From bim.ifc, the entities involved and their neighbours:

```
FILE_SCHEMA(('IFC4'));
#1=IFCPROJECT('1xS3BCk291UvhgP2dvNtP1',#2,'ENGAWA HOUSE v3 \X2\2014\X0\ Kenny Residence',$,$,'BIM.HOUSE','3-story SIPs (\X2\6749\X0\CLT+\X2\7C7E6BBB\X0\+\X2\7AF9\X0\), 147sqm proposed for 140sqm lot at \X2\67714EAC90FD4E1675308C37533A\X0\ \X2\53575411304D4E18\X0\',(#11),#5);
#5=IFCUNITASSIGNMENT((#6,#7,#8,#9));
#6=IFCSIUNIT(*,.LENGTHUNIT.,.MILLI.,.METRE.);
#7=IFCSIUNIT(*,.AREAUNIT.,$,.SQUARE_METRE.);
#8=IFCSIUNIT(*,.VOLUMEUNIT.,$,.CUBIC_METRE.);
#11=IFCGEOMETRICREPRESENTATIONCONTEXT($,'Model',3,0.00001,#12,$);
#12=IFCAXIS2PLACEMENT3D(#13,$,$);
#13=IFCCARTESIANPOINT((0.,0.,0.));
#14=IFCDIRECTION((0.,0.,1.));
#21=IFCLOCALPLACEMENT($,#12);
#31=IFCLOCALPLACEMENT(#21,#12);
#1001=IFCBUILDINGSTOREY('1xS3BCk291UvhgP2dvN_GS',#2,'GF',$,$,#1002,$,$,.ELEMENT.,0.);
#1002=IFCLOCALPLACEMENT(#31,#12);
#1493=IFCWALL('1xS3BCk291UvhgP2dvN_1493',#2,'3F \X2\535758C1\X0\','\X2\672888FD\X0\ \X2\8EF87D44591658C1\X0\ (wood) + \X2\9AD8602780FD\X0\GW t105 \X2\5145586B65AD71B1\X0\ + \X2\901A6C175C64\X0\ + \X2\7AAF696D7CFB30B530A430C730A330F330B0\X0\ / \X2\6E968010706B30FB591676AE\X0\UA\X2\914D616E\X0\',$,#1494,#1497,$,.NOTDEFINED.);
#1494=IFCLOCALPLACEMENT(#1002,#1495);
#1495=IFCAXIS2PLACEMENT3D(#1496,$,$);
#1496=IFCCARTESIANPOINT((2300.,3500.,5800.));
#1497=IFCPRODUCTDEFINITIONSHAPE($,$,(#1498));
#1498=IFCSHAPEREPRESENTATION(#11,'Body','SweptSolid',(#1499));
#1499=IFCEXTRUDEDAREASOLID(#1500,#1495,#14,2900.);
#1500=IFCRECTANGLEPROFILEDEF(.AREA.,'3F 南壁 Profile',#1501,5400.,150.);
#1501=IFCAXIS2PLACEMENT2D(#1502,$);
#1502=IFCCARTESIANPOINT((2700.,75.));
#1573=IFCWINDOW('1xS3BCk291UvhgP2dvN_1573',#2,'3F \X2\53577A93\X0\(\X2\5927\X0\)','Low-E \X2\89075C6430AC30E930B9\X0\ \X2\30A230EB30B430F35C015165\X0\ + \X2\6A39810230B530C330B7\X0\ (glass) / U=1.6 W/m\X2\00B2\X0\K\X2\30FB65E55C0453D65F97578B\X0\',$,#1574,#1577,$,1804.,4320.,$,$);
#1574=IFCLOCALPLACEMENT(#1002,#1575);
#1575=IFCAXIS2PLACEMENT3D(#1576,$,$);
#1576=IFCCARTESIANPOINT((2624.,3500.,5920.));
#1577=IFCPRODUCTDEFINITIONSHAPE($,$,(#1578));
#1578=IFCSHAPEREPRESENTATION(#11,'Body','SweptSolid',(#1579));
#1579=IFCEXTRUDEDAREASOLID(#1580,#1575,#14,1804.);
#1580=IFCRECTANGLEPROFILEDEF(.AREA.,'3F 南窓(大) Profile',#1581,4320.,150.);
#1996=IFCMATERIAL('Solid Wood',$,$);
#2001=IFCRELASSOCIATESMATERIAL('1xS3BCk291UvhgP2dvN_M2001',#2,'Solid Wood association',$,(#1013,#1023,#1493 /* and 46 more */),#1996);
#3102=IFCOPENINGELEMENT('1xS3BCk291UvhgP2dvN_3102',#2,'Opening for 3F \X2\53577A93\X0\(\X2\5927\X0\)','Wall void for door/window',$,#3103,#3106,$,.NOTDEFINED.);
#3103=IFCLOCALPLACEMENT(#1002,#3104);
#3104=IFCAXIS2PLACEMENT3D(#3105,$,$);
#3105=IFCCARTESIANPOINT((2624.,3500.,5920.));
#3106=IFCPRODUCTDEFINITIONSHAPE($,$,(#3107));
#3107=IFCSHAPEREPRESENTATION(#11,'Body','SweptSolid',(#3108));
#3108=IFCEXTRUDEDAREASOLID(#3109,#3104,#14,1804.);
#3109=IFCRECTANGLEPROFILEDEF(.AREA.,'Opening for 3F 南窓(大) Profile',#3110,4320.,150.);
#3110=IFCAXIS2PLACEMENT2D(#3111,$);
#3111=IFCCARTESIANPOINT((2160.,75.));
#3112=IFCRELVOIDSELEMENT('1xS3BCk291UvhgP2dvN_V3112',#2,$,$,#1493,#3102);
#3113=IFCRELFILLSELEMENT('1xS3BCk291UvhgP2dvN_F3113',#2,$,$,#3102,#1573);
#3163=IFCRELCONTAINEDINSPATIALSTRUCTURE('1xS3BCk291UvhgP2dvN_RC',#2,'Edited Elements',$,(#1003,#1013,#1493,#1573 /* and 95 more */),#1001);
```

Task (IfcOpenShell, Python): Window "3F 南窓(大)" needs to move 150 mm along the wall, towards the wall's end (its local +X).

```python
import ifcopenshell
import ifcopenshell.api.geometry
import ifcopenshell.util.placement

model = ifcopenshell.open("bim.ifc")

window = model.by_id(1573)
opening = window.FillsVoids[0].RelatingOpeningElement
wall = opening.VoidsElements[0].RelatingBuildingElement

wall_matrix = ifcopenshell.util.placement.get_local_placement(wall.ObjectPlacement)
shift = wall_matrix[:3, 0] * 150.0
before = ifcopenshell.util.placement.get_local_placement(window.ObjectPlacement)[:3, 3].copy()

# The window is not placed relative to its opening, so move both.
for product in (opening, window):
    matrix = ifcopenshell.util.placement.get_local_placement(product.ObjectPlacement)
    matrix[:3, 3] += shift
    ifcopenshell.api.geometry.edit_object_placement(model, product=product, matrix=matrix, is_si=False)

after = ifcopenshell.util.placement.get_local_placement(window.ObjectPlacement)[:3, 3]
print("window moved by", (after - before).round(3) + 0.0)

model.write("bim_edited.ifc")
```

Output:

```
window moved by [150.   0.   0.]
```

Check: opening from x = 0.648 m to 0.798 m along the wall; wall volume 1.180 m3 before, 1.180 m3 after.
